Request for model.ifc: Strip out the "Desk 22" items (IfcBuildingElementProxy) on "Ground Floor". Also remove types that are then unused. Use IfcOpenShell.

First a look at what the model holds.

```python
import ifcopenshell
import ifcopenshell.util.element

model = ifcopenshell.open("model.ifc")
print(model.schema)
storey = next(s for s in model.by_type("IfcBuildingStorey") if s.Name == "Ground Floor")
proxies = [e for e in ifcopenshell.util.element.get_decomposition(storey) if e.is_a("IfcBuildingElementProxy")]
seen = {}
for e in proxies:
    element_type = ifcopenshell.util.element.get_type(e)
    name = element_type.Name if element_type not in (None, e) else None
    seen[name] = seen.get(name, 0) + 1
for name, count in sorted(seen.items(), key=str):
    print(count, "x", name)
```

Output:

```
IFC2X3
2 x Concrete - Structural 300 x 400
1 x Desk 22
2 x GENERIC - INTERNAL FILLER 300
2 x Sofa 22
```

```python
import ifcopenshell
import ifcopenshell.api.root
import ifcopenshell.util.element

model = ifcopenshell.open("model.ifc")

storey = next(s for s in model.by_type("IfcBuildingStorey") if s.Name == "Ground Floor")
proxies = [e for e in ifcopenshell.util.element.get_decomposition(storey) if e.is_a("IfcBuildingElementProxy")]
targets = [e for e in proxies if (t := ifcopenshell.util.element.get_type(e)) not in (None, e) and t.Name == "Desk 22"]
types = {ifcopenshell.util.element.get_type(e) for e in targets} - {None, *targets}

for e in targets:
    ifcopenshell.api.root.remove_product(model, product=e)
print(len(targets), "removed")

unused = [t for t in types if not ifcopenshell.util.element.get_types(t)]
for t in unused:
    ifcopenshell.api.root.remove_product(model, product=t)
print(len(unused), "unused types removed")

model.write("model_edited.ifc")
```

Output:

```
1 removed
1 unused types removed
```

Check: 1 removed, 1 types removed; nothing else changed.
